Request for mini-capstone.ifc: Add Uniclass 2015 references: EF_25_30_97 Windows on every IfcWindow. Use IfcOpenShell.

First a look at what the model holds.

```python
import ifcopenshell

model = ifcopenshell.open("mini-capstone.ifc")
print(model.schema)
print("classifications:", [c.Name for c in model.by_type("IfcClassification")])
for ifc_class in ("IfcDoor", "IfcRoof", "IfcStair", "IfcWall", "IfcWindow"):
    print(ifc_class, len(model.by_type(ifc_class)))
```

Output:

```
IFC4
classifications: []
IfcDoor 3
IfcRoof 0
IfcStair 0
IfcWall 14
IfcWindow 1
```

```python
import ifcopenshell
import ifcopenshell.api.classification

model = ifcopenshell.open("mini-capstone.ifc")

system = ifcopenshell.api.classification.add_classification(model, classification="Uniclass 2015")

codes = {
    "IfcWindow": ("EF_25_30_97", "Windows"),
}
for ifc_class, (code, name) in codes.items():
    products = model.by_type(ifc_class)
    ifcopenshell.api.classification.add_reference(
        model, products=products, classification=system, identification=code, name=name
    )
    print(code, len(products))

model.write("mini-capstone_edited.ifc")
```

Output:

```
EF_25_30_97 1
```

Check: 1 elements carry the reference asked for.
